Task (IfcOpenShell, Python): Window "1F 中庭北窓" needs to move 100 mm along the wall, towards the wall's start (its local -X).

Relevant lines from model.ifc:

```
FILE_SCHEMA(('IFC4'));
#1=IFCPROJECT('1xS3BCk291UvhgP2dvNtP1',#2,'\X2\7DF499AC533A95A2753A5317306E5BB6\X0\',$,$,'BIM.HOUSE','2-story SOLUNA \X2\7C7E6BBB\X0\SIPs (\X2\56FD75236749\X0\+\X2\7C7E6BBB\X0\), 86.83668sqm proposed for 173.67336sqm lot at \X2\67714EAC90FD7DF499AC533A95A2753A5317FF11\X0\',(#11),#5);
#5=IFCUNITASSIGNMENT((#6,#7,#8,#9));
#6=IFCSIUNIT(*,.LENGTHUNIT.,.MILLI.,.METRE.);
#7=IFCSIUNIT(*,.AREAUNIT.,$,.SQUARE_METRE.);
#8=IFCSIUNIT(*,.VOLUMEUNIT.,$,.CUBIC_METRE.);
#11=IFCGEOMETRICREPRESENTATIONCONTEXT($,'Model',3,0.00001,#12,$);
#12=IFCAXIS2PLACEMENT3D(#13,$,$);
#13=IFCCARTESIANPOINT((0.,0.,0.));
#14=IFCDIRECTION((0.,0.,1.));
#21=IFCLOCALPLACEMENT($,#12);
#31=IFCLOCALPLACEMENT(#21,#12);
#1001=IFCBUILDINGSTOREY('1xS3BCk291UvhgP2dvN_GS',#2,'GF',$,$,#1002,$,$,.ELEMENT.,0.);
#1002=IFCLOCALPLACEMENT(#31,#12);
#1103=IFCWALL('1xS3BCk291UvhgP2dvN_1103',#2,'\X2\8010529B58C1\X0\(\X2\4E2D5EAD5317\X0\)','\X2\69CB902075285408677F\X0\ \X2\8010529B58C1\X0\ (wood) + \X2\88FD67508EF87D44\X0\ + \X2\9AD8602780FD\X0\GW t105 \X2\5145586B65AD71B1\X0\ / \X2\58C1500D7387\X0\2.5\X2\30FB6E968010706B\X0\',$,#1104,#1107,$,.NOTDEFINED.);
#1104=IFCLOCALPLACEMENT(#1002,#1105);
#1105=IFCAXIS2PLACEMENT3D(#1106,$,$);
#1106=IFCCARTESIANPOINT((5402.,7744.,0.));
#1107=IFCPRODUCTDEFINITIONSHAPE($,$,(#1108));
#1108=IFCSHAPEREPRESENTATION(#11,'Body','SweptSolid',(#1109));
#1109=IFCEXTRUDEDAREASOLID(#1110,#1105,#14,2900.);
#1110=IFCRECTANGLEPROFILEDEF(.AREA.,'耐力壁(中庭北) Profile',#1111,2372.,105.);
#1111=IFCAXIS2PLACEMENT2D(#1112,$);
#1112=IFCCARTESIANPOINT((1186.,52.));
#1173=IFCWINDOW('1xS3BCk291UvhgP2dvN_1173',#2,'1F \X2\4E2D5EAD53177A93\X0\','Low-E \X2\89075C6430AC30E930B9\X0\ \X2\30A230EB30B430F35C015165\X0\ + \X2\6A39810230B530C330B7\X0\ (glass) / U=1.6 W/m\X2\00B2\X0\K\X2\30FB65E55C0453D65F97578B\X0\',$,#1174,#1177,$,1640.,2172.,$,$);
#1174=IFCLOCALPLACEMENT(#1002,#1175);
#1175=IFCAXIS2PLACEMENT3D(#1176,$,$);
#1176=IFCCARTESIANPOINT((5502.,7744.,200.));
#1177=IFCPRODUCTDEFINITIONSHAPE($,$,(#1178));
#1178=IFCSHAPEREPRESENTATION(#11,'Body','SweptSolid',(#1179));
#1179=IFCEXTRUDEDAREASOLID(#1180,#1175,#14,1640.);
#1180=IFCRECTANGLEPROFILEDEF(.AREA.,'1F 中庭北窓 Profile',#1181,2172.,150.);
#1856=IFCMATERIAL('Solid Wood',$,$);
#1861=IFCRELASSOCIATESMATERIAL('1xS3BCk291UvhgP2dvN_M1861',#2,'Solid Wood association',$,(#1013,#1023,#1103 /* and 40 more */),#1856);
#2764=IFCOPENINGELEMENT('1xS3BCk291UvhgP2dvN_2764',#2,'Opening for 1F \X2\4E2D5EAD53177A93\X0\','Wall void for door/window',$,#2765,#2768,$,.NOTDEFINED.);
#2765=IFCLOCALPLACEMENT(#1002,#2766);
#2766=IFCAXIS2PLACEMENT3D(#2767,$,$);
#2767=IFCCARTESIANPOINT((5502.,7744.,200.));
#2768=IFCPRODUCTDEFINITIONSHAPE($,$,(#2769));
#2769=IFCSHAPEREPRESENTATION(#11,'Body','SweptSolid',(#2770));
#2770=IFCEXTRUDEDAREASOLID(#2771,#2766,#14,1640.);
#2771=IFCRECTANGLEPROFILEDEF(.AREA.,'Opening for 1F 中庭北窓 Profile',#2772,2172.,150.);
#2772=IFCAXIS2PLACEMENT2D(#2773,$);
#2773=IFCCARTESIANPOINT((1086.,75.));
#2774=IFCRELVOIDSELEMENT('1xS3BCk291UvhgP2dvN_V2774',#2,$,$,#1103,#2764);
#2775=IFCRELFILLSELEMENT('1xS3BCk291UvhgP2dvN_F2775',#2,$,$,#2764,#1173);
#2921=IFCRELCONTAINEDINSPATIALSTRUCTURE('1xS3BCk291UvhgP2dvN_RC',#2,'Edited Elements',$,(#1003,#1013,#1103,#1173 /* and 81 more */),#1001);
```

```python
import ifcopenshell
import ifcopenshell.api.geometry
import ifcopenshell.util.placement
import ifcopenshell.util.unit

model = ifcopenshell.open("model.ifc")
unit_scale = ifcopenshell.util.unit.calculate_unit_scale(model)

window = model.by_guid("1xS3BCk291UvhgP2dvN_1173")
opening = window.FillsVoids[0].RelatingOpeningElement
wall = opening.VoidsElements[0].RelatingBuildingElement

wall_matrix = ifcopenshell.util.placement.get_local_placement(wall.ObjectPlacement)
shift = wall_matrix[:3, 0] * -0.1 / unit_scale
before = ifcopenshell.util.placement.get_local_placement(window.ObjectPlacement)[:3, 3].copy()

# The window is not placed relative to its opening, so move both.
for product in (opening, window):
    matrix = ifcopenshell.util.placement.get_local_placement(product.ObjectPlacement)
    matrix[:3, 3] += shift
    ifcopenshell.api.geometry.edit_object_placement(model, product=product, matrix=matrix, is_si=False)

after = ifcopenshell.util.placement.get_local_placement(window.ObjectPlacement)[:3, 3]
print("window moved by", (after - before).round(3) + 0.0)

model.write("model-out.ifc")
```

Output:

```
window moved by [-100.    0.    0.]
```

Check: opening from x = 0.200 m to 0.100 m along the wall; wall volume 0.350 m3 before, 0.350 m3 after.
